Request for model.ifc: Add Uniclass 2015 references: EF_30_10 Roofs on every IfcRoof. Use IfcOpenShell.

First a look at what the model holds.

```python
import ifcopenshell

model = ifcopenshell.open("model.ifc")
print(model.schema)
print("classifications:", [c.Name for c in model.by_type("IfcClassification")])
for ifc_class in ("IfcDoor", "IfcRoof", "IfcStair", "IfcWall", "IfcWindow"):
    print(ifc_class, len(model.by_type(ifc_class)))
```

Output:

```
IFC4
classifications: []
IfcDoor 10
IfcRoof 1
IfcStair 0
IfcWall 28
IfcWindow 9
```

```python
import ifcopenshell
import ifcopenshell.api.classification

model = ifcopenshell.open("model.ifc")

system = ifcopenshell.api.classification.add_classification(model, classification="Uniclass 2015")

codes = {
    "IfcRoof": ("EF_30_10", "Roofs"),
}
for ifc_class, (code, name) in codes.items():
    products = model.by_type(ifc_class)
    ifcopenshell.api.classification.add_reference(
        model, products=products, classification=system, identification=code, name=name
    )
    print(code, len(products))

model.write("model_v2.ifc")
```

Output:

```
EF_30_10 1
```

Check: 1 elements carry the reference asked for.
